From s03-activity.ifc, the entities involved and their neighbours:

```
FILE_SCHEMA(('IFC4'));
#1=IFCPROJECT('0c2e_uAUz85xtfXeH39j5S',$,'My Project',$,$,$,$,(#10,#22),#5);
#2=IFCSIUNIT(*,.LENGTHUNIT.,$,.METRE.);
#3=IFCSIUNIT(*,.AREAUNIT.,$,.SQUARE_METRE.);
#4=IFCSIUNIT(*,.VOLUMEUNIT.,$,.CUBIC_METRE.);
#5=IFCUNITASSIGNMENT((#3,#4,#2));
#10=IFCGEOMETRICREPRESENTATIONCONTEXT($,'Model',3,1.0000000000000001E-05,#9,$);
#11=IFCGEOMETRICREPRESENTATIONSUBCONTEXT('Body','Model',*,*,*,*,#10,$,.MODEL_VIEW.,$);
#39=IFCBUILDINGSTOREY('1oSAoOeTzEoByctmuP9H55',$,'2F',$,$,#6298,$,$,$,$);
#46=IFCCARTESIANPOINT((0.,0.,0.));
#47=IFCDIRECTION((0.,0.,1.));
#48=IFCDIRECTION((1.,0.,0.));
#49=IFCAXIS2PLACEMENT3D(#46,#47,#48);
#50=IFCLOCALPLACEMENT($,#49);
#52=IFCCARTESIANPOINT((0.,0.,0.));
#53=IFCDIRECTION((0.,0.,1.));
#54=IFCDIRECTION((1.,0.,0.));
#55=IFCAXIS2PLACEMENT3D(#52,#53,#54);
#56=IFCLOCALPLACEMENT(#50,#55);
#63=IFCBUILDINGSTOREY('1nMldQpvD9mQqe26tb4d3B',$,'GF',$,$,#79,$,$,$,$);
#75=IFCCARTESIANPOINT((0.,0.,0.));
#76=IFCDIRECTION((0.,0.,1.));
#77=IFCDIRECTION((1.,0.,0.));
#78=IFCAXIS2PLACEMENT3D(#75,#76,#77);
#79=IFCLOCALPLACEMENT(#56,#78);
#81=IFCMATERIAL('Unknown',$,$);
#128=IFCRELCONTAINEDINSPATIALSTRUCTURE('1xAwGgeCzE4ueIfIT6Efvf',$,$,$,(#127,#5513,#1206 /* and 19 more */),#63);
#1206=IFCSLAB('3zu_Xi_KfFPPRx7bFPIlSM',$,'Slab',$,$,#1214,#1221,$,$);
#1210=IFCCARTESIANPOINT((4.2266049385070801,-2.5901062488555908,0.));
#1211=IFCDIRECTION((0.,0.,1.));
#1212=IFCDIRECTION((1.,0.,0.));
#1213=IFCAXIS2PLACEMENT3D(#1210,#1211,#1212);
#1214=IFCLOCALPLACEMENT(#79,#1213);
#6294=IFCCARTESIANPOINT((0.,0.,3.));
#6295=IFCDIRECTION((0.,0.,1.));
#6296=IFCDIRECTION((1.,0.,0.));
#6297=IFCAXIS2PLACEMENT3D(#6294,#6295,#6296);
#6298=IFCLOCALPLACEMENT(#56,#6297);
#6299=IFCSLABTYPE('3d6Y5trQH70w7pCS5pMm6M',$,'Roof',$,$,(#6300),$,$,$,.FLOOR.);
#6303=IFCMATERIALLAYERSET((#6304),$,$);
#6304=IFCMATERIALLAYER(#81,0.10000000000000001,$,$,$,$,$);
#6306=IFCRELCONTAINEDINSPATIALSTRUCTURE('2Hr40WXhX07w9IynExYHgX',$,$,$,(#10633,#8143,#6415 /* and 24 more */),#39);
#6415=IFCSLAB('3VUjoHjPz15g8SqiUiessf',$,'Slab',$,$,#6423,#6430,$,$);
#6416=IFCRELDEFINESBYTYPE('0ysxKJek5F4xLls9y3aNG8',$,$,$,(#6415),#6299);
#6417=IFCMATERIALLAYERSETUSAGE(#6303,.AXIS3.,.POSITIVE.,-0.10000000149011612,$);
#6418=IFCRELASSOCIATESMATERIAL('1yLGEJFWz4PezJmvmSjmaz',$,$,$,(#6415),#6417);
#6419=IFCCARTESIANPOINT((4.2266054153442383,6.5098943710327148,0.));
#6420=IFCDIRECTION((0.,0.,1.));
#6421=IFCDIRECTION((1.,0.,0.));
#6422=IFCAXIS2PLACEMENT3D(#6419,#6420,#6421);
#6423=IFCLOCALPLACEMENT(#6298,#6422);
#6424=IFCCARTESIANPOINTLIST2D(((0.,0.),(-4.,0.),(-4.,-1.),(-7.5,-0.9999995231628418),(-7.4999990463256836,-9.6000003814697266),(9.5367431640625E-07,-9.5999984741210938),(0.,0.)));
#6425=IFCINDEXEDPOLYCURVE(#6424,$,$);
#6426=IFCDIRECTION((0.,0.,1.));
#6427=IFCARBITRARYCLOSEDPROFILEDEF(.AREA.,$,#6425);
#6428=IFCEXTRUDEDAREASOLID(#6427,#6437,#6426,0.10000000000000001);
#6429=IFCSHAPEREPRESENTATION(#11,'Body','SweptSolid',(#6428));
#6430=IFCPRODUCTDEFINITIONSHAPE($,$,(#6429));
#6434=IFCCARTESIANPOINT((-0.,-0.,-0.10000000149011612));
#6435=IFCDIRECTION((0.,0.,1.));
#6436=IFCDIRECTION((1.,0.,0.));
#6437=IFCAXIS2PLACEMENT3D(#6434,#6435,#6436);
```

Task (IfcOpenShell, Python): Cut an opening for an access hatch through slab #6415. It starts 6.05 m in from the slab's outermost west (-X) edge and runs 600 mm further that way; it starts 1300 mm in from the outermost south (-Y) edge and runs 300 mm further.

```python
import numpy as np
import ifcopenshell
import ifcopenshell.api.feature
import ifcopenshell.api.geometry
import ifcopenshell.api.root
import ifcopenshell.geom
import ifcopenshell.util.placement
import ifcopenshell.util.representation
import ifcopenshell.util.shape
import ifcopenshell.util.unit

model = ifcopenshell.open("s03-activity.ifc")
unit_scale = ifcopenshell.util.unit.calculate_unit_scale(model)
settings = ifcopenshell.geom.settings()


def volume(element):
    """Net volume in cubic metres, openings subtracted."""
    shape = ifcopenshell.geom.create_shape(settings, element)
    return ifcopenshell.util.shape.get_volume(shape.geometry)


slab = model.by_guid("3VUjoHjPz15g8SqiUiessf")
before = volume(slab)

# Extent in the slab's own axes, in metres. The edges named are its -X and -Y sides.
slab_shape = ifcopenshell.geom.create_shape(settings, slab)
vertices = ifcopenshell.util.shape.get_vertices(slab_shape.geometry)
x_min, y_min, bottom = vertices.min(axis=0)
top = vertices[:, 2].max()

opening = ifcopenshell.api.root.create_entity(model, ifc_class="IfcOpeningElement", name="Access hatch opening", predefined_type="OPENING")
context = ifcopenshell.util.representation.get_context(model, "Model", "Body", "MODEL_VIEW")
width, depth = 0.6, 0.3
outline = [(0.0, 0.0), (width, 0.0), (width, depth), (0.0, depth), (0.0, 0.0)]
# Overshoot both faces by 50 mm so the cut is clean.
shape = ifcopenshell.api.geometry.add_slab_representation(
    model, context=context, depth=top - bottom + 0.1, polyline=outline
)
ifcopenshell.api.geometry.assign_representation(model, product=opening, representation=shape)

matrix = ifcopenshell.util.placement.get_local_placement(slab.ObjectPlacement)
matrix[:, 3] = matrix @ np.append(np.array([x_min + 6.05, y_min + 1.3, bottom - 0.05]) / unit_scale, 1.0)
ifcopenshell.api.geometry.edit_object_placement(model, product=opening, matrix=matrix, is_si=False)
ifcopenshell.api.feature.add_feature(model, feature=opening, element=slab)

after = volume(slab)

print(f"slab volume {before:.3f} -> {after:.3f} m3")

model.write("s03-activity_edited.ifc")
```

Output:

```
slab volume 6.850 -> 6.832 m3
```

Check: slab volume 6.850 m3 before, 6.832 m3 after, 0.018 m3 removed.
